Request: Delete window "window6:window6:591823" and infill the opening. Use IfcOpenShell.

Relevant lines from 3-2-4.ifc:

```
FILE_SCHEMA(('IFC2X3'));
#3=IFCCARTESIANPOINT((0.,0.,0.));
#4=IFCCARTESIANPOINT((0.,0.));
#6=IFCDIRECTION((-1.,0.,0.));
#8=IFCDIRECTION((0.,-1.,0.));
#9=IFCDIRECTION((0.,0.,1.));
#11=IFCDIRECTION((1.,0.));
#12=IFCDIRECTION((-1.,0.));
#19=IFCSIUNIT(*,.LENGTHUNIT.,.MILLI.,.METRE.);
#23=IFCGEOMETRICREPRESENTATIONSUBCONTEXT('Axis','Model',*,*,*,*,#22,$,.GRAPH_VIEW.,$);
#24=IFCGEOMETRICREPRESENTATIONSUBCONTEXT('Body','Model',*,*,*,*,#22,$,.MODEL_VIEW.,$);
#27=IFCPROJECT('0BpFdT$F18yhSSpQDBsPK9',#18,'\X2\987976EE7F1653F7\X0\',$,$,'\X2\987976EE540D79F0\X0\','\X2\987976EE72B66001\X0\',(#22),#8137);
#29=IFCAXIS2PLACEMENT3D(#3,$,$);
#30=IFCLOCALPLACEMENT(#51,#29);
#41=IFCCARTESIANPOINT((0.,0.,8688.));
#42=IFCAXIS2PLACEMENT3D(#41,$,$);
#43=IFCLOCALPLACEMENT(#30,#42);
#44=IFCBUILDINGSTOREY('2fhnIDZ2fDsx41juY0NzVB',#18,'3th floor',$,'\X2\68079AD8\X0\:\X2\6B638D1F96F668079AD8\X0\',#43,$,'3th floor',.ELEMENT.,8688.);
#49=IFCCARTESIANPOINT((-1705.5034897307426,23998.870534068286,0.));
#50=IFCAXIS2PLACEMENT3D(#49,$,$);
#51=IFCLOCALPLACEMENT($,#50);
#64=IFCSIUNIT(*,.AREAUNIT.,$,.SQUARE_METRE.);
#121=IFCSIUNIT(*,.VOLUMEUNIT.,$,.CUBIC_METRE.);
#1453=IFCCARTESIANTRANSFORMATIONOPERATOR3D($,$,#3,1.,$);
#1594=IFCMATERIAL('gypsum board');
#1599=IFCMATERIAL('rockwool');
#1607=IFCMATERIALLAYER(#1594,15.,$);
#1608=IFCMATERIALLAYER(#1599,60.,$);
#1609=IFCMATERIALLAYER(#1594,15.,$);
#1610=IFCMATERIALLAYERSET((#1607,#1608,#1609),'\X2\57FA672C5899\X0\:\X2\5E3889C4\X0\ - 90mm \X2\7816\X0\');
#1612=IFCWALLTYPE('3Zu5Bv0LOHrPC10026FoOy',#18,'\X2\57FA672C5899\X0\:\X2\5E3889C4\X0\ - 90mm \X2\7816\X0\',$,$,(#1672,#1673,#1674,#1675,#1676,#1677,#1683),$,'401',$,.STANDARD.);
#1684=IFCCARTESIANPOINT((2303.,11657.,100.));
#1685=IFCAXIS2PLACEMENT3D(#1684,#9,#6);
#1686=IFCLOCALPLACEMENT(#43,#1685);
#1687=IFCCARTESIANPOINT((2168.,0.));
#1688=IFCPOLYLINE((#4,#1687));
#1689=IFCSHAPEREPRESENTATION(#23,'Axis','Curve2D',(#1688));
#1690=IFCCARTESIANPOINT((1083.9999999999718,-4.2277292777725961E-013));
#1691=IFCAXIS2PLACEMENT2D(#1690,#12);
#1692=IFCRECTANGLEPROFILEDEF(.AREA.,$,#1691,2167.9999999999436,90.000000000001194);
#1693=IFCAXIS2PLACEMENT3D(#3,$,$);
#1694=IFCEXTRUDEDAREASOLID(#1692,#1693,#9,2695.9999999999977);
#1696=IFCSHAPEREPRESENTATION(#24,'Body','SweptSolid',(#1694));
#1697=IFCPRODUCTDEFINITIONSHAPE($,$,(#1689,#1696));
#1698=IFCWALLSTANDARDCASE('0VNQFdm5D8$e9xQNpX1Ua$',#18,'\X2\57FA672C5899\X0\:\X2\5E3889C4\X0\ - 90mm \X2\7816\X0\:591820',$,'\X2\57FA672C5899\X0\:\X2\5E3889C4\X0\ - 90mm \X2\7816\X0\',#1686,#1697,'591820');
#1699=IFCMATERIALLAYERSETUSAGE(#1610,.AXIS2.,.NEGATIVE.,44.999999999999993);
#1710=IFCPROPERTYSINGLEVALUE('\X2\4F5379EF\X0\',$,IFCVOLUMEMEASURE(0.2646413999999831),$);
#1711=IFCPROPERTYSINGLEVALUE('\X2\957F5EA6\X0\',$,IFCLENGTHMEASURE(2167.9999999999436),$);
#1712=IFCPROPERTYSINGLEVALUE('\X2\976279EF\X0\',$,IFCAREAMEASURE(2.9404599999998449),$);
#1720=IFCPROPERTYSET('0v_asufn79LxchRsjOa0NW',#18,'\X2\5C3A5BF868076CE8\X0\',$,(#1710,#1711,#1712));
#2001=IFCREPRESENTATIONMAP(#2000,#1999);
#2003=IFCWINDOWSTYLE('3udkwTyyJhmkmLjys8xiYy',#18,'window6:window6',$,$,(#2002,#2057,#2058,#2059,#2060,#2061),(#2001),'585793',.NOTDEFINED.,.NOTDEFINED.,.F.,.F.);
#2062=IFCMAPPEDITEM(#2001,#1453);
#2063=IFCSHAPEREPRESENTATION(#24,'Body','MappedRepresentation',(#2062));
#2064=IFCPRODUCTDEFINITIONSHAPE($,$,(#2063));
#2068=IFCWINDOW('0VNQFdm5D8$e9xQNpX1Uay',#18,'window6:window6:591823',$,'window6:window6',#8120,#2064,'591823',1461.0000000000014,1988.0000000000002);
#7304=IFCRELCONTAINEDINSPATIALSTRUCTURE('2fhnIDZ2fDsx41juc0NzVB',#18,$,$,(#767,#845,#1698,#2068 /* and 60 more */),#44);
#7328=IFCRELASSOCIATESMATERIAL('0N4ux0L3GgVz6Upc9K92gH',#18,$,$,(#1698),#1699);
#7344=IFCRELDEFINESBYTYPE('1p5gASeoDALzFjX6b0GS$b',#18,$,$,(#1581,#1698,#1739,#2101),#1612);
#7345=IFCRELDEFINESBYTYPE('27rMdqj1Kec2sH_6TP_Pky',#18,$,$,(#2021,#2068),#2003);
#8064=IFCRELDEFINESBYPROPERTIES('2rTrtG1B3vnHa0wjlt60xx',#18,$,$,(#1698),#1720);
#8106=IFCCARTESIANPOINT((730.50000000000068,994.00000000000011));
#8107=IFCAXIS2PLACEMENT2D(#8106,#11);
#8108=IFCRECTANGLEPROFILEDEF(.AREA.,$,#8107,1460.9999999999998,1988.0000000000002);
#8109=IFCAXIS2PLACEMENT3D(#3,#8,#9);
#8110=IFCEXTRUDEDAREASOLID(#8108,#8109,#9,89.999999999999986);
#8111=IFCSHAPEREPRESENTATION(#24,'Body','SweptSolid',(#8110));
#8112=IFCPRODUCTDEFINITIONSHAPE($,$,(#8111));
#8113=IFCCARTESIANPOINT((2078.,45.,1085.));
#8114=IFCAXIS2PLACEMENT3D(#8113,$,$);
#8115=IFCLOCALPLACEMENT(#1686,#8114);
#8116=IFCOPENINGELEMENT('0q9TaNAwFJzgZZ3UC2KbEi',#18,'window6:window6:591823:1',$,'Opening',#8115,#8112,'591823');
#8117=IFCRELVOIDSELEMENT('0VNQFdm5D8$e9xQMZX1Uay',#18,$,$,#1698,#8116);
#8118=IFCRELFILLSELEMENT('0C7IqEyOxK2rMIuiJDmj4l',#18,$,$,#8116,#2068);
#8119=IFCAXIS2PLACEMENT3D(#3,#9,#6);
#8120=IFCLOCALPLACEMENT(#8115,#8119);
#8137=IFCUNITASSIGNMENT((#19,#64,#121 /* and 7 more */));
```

```python
import ifcopenshell
import ifcopenshell.api.feature
import ifcopenshell.api.pset
import ifcopenshell.api.root
import ifcopenshell.geom
import ifcopenshell.util.element
import ifcopenshell.util.shape
import ifcopenshell.util.unit

model = ifcopenshell.open("3-2-4.ifc")
area_scale = ifcopenshell.util.unit.calculate_unit_scale(model, "AREAUNIT")
volume_scale = ifcopenshell.util.unit.calculate_unit_scale(model, "VOLUMEUNIT")
settings = ifcopenshell.geom.settings()


def volume(element):
    """Net volume in cubic metres, openings subtracted."""
    shape = ifcopenshell.geom.create_shape(settings, element)
    return ifcopenshell.util.shape.get_volume(shape.geometry)


window = model.by_guid("0VNQFdm5D8$e9xQNpX1Uay")
opening = window.FillsVoids[0].RelatingOpeningElement
wall = opening.VoidsElements[0].RelatingBuildingElement
before = volume(wall)

ifcopenshell.api.root.remove_product(model, product=window)
ifcopenshell.api.feature.remove_feature(model, feature=opening)

after = volume(wall)
thickness = 0.09  # wall thickness in metres

# Update the wall's stored quantities.
pset = model.by_id(ifcopenshell.util.element.get_pset(wall, "尺寸标注", should_inherit=False)["id"])
ifcopenshell.api.pset.edit_pset(model, pset=pset, properties={
    "体积": model.create_entity("IfcVolumeMeasure", after / volume_scale),
    "面积": model.create_entity("IfcAreaMeasure", after / thickness / area_scale),
})

print(f"wall volume {before:.3f} -> {after:.3f} m3")

model.write("3-2-4-out.ifc")
```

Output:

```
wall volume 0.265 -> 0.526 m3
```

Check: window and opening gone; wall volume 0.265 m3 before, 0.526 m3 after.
